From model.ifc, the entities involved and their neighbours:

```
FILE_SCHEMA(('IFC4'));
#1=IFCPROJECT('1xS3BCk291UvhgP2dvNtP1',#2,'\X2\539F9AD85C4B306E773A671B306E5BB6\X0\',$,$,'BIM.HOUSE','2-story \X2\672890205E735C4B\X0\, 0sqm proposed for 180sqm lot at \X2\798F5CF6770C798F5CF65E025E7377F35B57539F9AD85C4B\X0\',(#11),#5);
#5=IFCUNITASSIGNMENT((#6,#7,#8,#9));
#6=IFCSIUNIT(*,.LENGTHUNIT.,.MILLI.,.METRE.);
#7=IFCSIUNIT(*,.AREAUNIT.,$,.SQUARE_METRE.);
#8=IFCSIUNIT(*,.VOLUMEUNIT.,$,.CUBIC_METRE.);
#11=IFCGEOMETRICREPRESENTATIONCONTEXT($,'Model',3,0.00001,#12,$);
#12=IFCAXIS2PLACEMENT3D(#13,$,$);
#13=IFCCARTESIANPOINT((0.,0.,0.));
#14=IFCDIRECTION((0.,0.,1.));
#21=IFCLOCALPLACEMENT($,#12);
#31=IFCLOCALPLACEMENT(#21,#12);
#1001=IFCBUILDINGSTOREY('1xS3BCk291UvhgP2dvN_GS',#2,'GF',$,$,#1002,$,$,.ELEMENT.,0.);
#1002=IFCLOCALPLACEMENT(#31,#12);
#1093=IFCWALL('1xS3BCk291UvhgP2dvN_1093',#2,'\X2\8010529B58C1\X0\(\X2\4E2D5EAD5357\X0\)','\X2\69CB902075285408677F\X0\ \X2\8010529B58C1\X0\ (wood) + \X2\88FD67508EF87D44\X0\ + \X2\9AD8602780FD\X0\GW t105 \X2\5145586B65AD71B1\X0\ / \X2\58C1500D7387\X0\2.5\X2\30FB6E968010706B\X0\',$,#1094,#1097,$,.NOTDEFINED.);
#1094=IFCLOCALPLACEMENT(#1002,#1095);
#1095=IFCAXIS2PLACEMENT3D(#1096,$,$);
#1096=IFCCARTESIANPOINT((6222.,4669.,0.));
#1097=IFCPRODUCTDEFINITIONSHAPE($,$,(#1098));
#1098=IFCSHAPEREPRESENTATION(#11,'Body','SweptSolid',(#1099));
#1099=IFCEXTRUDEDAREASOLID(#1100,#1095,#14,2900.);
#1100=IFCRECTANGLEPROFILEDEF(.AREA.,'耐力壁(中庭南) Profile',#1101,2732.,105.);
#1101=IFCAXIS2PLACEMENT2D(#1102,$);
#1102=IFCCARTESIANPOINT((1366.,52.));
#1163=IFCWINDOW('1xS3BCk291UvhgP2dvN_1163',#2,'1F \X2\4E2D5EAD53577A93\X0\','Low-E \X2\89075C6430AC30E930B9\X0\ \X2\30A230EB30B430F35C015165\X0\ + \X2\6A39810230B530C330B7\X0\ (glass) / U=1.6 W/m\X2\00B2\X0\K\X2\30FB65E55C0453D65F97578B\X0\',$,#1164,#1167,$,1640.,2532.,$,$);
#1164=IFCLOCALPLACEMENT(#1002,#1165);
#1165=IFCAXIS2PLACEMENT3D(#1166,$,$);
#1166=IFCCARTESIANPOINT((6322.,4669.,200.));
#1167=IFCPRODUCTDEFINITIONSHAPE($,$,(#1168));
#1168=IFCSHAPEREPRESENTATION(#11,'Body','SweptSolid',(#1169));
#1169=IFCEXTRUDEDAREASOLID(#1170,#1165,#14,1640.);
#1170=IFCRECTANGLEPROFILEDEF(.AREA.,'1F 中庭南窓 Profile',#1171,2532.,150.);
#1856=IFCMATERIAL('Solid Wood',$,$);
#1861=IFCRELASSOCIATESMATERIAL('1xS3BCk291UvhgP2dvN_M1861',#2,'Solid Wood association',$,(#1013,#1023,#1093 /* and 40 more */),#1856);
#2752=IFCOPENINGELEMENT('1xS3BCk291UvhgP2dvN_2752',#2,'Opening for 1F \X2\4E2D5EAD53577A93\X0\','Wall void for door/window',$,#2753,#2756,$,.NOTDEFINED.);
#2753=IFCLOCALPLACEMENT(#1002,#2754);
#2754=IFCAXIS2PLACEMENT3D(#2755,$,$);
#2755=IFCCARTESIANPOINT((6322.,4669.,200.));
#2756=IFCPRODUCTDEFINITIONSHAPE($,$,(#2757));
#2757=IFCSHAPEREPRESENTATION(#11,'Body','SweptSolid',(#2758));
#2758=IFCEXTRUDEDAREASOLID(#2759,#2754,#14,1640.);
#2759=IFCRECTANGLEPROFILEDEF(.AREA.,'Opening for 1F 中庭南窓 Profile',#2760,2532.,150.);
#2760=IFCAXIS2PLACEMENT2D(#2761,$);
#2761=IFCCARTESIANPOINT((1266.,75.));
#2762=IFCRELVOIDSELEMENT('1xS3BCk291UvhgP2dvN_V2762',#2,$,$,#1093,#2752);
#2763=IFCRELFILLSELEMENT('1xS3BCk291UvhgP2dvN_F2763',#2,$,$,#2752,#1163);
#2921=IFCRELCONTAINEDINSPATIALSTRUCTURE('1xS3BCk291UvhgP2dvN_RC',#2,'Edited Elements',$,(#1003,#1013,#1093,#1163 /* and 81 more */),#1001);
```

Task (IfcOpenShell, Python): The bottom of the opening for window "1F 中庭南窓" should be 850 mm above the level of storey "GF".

```python
import numpy as np
import ifcopenshell
import ifcopenshell.api.geometry
import ifcopenshell.geom
import ifcopenshell.util.element
import ifcopenshell.util.placement
import ifcopenshell.util.shape
import ifcopenshell.util.unit

model = ifcopenshell.open("model.ifc")
unit_scale = ifcopenshell.util.unit.calculate_unit_scale(model)

window = model.by_guid("1xS3BCk291UvhgP2dvN_1163")
opening = window.FillsVoids[0].RelatingOpeningElement
storey = ifcopenshell.util.element.get_container(window, ifc_class="IfcBuildingStorey")
level = ifcopenshell.util.placement.get_local_placement(storey.ObjectPlacement)[2, 3]

# The opening's origin need not be at the sill, so measure its lowest point.
shape = ifcopenshell.geom.create_shape(ifcopenshell.geom.settings(), opening)
bottom = ifcopenshell.util.shape.get_shape_bottom_elevation(shape, shape.geometry) / unit_scale
dz = level + 0.85 / unit_scale - bottom

shift = np.array([0.0, 0.0, dz])
# The window is not placed relative to its opening, so move both.
for product in (opening, window):
    matrix = ifcopenshell.util.placement.get_local_placement(product.ObjectPlacement)
    matrix[:3, 3] += shift
    ifcopenshell.api.geometry.edit_object_placement(model, product=product, matrix=matrix, is_si=False)

print(f"moved by {dz * unit_scale:+.3f} m")

model.write("model_rev.ifc")
```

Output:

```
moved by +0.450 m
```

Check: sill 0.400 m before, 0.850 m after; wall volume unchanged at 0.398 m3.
